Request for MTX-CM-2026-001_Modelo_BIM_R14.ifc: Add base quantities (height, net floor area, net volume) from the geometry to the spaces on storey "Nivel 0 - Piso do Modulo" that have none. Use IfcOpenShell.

First a look at what the model holds.

```python
import ifcopenshell
import ifcopenshell.util.element
import ifcopenshell.util.unit

model = ifcopenshell.open("MTX-CM-2026-001_Modelo_BIM_R14.ifc")
print(model.schema)
for unit_type in ("LENGTHUNIT", "AREAUNIT", "VOLUMEUNIT"):
    print(unit_type, ifcopenshell.util.unit.calculate_unit_scale(model, unit_type))
storey = next(s for s in model.by_type("IfcBuildingStorey") if s.Name == "Nivel 0 - Piso do Modulo")
spaces = [e for e in ifcopenshell.util.element.get_decomposition(storey) if e.is_a("IfcSpace")]
for e in sorted(spaces, key=lambda e: e.id()):
    print(e.id(), e.is_a(), e.Name, list(ifcopenshell.util.element.get_psets(e, qtos_only=True)), sep=" | ")
```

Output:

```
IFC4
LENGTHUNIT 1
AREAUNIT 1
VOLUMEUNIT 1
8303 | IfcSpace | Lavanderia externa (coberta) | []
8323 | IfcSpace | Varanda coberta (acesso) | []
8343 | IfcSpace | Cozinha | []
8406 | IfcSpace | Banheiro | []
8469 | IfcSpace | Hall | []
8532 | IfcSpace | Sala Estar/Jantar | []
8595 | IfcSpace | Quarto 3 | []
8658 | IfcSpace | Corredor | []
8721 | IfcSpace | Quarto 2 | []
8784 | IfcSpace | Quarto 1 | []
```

```python
import ifcopenshell
import ifcopenshell.api.pset
import ifcopenshell.geom
import ifcopenshell.util.element
import ifcopenshell.util.shape
import ifcopenshell.util.unit

model = ifcopenshell.open("MTX-CM-2026-001_Modelo_BIM_R14.ifc")
unit_scale = ifcopenshell.util.unit.calculate_unit_scale(model)
area_scale = ifcopenshell.util.unit.calculate_unit_scale(model, "AREAUNIT")
volume_scale = ifcopenshell.util.unit.calculate_unit_scale(model, "VOLUMEUNIT")
settings = ifcopenshell.geom.settings()

storey = next(s for s in model.by_type("IfcBuildingStorey") if s.Name == "Nivel 0 - Piso do Modulo")
spaces = [e for e in ifcopenshell.util.element.get_decomposition(storey) if e.is_a("IfcSpace")]

for e in sorted(spaces, key=lambda e: e.id()):
    if ifcopenshell.util.element.get_psets(e, qtos_only=True, should_inherit=False):
        continue
    # Geometry comes back in metres, in the element's own axes.
    shape = ifcopenshell.geom.create_shape(settings, e)
    values = {
        "Height": ifcopenshell.util.shape.get_z(shape.geometry) / unit_scale,
        "NetFloorArea": ifcopenshell.util.shape.get_footprint_area(shape.geometry) / area_scale,
        "NetVolume": ifcopenshell.util.shape.get_volume(shape.geometry) / volume_scale,
    }
    qto = ifcopenshell.api.pset.add_qto(model, product=e, name="Qto_SpaceBaseQuantities")
    ifcopenshell.api.pset.edit_qto(model, qto=qto, properties=values)
    print(e.id(), {k: round(v, 3) for k, v in values.items()})

model.write("MTX-CM-2026-001_Modelo_BIM_R14_updated.ifc")
```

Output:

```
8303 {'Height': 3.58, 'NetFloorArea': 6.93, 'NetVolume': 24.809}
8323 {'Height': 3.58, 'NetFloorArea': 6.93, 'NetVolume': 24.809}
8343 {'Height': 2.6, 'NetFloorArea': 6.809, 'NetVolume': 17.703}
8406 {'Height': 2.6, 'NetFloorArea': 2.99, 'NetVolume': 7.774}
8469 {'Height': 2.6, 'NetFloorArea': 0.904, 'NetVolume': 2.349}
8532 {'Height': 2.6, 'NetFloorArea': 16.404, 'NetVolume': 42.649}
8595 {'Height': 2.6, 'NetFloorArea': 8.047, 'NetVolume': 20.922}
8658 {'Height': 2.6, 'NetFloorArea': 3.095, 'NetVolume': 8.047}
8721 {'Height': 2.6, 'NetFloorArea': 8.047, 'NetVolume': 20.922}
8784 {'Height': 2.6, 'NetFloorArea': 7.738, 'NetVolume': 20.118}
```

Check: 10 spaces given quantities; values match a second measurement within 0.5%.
